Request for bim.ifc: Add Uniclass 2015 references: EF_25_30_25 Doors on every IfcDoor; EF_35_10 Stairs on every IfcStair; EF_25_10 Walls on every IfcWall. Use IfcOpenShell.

First a look at what the model holds.

```python
import ifcopenshell

model = ifcopenshell.open("bim.ifc")
print(model.schema)
print("classifications:", [c.Name for c in model.by_type("IfcClassification")])
for ifc_class in ("IfcDoor", "IfcRoof", "IfcStair", "IfcWall", "IfcWindow"):
    print(ifc_class, len(model.by_type(ifc_class)))
```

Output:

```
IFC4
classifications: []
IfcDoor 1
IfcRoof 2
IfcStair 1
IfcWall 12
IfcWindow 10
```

```python
import ifcopenshell
import ifcopenshell.api.classification

model = ifcopenshell.open("bim.ifc")

system = ifcopenshell.api.classification.add_classification(model, classification="Uniclass 2015")

codes = {
    "IfcDoor": ("EF_25_30_25", "Doors"),
    "IfcStair": ("EF_35_10", "Stairs"),
    "IfcWall": ("EF_25_10", "Walls"),
}
for ifc_class, (code, name) in codes.items():
    products = model.by_type(ifc_class)
    ifcopenshell.api.classification.add_reference(
        model, products=products, classification=system, identification=code, name=name
    )
    print(code, len(products))

model.write("bim_v2.ifc")
```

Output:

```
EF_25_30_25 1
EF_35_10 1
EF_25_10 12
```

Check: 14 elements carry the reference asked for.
